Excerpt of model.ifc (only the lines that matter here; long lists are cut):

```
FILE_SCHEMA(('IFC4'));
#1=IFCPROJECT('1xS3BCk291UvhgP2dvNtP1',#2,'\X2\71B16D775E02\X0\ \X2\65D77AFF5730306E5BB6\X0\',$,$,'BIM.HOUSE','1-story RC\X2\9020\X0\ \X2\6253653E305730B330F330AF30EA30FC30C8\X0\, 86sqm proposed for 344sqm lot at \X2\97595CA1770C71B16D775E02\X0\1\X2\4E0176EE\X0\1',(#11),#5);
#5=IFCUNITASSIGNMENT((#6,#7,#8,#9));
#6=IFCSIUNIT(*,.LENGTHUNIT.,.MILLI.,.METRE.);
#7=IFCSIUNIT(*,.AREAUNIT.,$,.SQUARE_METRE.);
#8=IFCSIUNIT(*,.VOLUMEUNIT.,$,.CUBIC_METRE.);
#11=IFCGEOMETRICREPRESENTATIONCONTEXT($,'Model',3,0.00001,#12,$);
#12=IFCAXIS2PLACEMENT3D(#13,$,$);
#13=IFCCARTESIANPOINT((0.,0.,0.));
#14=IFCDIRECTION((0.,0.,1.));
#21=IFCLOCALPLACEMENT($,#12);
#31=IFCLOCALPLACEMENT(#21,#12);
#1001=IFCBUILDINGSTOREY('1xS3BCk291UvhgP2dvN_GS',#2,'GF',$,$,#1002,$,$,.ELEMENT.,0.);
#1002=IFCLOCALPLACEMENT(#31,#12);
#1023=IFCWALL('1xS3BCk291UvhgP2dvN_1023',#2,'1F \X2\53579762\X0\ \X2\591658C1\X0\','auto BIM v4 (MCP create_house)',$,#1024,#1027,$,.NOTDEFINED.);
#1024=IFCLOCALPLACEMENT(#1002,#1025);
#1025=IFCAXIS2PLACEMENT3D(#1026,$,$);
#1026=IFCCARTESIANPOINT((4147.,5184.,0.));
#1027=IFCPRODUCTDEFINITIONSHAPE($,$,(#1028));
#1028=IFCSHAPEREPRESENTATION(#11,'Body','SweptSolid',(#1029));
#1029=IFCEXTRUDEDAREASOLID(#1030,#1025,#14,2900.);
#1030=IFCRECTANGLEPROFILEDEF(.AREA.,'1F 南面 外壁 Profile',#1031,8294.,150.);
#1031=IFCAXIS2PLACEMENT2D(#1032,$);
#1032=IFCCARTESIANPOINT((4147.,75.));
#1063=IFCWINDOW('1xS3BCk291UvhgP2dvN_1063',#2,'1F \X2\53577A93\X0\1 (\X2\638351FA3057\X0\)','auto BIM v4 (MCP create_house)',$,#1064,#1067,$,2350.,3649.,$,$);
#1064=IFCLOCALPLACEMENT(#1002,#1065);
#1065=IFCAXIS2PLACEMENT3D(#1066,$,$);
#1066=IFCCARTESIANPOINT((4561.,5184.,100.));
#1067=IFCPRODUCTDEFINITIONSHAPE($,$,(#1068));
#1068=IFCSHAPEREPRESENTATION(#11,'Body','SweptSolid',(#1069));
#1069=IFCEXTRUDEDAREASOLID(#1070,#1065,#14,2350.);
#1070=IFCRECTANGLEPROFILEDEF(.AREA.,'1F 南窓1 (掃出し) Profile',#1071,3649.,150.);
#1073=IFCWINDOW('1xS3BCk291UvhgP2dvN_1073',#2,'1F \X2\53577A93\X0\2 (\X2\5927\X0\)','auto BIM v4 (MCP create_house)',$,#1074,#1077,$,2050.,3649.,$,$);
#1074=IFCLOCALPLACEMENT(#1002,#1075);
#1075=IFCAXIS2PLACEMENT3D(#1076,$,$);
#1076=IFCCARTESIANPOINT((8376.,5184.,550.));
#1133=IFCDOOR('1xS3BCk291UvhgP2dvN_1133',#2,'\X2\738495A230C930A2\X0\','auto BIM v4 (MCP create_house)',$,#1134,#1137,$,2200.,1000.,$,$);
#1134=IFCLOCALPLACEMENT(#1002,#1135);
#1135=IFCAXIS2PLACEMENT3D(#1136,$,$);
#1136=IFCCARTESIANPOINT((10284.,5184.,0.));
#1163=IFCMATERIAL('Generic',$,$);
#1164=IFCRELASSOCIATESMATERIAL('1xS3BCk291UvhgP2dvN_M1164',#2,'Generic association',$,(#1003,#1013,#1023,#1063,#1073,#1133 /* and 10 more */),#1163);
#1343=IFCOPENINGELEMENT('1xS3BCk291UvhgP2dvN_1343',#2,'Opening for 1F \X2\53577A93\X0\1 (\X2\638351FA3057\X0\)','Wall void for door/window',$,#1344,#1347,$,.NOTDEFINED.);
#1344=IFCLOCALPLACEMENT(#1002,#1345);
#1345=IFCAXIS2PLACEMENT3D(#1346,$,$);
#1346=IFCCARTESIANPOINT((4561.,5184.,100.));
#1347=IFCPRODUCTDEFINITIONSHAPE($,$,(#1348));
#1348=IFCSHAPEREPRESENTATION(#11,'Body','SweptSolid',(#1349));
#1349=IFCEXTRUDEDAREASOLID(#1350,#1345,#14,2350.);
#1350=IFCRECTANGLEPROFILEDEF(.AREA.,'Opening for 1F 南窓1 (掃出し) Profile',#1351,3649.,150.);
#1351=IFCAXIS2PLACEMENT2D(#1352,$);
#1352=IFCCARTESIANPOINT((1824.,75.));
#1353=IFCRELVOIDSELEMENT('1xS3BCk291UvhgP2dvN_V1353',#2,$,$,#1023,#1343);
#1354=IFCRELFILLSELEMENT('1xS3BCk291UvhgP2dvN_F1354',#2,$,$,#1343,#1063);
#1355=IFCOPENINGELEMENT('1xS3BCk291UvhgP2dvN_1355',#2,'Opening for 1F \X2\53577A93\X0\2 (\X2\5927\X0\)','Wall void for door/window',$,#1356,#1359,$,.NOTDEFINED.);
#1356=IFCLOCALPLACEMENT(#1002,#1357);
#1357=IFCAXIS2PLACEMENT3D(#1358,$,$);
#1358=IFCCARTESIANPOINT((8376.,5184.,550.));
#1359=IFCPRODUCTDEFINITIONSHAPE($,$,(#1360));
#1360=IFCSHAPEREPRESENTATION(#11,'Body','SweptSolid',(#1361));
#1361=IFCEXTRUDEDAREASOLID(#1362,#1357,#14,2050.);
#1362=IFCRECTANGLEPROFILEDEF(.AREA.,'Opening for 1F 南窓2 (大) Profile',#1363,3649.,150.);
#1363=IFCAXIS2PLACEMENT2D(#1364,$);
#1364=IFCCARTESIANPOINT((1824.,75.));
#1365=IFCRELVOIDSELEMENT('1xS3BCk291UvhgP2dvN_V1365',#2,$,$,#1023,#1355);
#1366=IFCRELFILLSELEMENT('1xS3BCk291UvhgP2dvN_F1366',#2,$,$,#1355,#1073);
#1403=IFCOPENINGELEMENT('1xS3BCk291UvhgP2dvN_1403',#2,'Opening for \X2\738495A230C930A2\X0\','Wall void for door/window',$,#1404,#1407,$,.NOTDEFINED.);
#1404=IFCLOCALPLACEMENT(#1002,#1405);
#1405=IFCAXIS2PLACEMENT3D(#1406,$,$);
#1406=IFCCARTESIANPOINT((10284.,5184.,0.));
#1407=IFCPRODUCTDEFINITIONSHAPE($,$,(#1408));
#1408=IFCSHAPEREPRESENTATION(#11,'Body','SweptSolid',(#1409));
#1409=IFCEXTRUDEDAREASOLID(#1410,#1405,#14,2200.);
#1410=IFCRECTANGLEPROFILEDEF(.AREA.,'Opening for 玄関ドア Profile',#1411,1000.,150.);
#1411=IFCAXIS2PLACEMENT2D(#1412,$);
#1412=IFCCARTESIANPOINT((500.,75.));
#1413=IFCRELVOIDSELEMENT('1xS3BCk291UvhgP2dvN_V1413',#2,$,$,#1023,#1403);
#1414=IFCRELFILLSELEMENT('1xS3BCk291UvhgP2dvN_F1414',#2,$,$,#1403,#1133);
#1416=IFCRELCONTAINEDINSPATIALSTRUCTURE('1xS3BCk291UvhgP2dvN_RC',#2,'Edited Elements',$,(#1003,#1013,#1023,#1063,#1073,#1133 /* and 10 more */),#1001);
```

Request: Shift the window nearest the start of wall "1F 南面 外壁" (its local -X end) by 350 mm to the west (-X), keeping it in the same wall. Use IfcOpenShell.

```python
import ifcopenshell
import ifcopenshell.api.geometry
import ifcopenshell.util.placement

model = ifcopenshell.open("model.ifc")

window = model.by_guid("1xS3BCk291UvhgP2dvN_1063")
opening = window.FillsVoids[0].RelatingOpeningElement
wall = opening.VoidsElements[0].RelatingBuildingElement

wall_matrix = ifcopenshell.util.placement.get_local_placement(wall.ObjectPlacement)
shift = wall_matrix[:3, 0] * -350.0
before = ifcopenshell.util.placement.get_local_placement(window.ObjectPlacement)[:3, 3].copy()

# The window is not placed relative to its opening, so move both.
for product in (opening, window):
    matrix = ifcopenshell.util.placement.get_local_placement(product.ObjectPlacement)
    matrix[:3, 3] += shift
    ifcopenshell.api.geometry.edit_object_placement(model, product=product, matrix=matrix, is_si=False)

after = ifcopenshell.util.placement.get_local_placement(window.ObjectPlacement)[:3, 3]
print("window moved by", (after - before).round(3) + 0.0)

model.write("model_edited.ifc")
```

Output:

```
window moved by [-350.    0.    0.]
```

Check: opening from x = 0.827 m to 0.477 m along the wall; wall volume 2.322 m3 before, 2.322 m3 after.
